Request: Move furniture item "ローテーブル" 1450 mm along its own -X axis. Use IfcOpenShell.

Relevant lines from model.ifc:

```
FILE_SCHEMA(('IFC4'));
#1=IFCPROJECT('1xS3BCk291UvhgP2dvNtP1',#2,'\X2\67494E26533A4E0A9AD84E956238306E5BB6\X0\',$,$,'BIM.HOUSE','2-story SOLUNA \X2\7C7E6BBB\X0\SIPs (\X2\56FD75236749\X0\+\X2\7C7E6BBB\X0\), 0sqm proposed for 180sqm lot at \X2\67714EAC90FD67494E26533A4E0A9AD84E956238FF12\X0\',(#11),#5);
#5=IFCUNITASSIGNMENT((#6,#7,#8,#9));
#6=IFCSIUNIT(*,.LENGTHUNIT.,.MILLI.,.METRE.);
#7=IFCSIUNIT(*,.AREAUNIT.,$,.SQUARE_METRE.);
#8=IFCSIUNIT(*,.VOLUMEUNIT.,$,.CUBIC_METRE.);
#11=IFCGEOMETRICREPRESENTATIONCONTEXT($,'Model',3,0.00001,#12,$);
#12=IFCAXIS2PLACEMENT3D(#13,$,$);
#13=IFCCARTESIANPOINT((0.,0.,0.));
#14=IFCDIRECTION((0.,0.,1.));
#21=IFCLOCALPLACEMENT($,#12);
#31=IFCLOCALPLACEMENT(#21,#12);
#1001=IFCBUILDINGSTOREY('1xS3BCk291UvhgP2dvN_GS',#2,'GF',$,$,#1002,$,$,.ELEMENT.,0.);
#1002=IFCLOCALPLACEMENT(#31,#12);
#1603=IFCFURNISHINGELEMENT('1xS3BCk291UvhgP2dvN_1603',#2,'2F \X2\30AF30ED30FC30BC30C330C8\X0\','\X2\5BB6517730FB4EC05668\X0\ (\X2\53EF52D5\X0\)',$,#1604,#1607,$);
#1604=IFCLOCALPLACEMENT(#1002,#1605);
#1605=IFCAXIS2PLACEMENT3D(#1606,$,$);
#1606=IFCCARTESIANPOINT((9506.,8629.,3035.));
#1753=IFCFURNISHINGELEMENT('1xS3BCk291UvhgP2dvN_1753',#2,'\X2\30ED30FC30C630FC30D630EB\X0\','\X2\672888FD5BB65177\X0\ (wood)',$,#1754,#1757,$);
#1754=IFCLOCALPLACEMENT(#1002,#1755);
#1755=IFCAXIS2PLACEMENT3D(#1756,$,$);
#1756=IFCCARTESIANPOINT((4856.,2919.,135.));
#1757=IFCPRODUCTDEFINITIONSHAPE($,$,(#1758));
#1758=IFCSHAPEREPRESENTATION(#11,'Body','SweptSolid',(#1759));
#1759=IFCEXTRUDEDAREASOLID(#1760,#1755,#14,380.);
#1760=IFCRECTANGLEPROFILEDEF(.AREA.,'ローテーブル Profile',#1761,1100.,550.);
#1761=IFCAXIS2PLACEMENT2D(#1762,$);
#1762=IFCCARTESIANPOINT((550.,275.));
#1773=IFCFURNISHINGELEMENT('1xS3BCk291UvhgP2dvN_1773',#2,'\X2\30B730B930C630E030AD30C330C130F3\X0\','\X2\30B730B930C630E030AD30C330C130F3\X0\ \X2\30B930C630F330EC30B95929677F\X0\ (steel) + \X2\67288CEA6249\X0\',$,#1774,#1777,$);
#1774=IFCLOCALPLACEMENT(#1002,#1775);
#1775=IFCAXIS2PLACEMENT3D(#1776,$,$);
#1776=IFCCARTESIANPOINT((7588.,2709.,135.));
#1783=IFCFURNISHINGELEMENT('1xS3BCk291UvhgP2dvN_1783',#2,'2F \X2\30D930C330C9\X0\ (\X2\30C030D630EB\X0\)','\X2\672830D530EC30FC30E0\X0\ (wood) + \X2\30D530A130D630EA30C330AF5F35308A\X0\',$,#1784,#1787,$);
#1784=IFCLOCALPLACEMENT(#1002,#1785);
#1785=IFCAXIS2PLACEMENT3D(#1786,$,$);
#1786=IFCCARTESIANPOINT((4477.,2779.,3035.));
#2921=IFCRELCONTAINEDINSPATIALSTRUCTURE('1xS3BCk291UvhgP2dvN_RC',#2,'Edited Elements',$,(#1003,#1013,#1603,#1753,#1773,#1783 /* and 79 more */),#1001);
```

```python
import ifcopenshell
import ifcopenshell.api.geometry
import ifcopenshell.util.placement
import ifcopenshell.util.unit

model = ifcopenshell.open("model.ifc")
unit_scale = ifcopenshell.util.unit.calculate_unit_scale(model)

item = model.by_guid("1xS3BCk291UvhgP2dvN_1753")
matrix = ifcopenshell.util.placement.get_local_placement(item.ObjectPlacement)
matrix[:3, 3] -= matrix[:3, 0] * 1.45 / unit_scale
ifcopenshell.api.geometry.edit_object_placement(model, product=item, matrix=matrix, is_si=False)

print(ifcopenshell.util.placement.get_local_placement(item.ObjectPlacement).round(3) + 0.0)

model.write("model_edited.ifc")
```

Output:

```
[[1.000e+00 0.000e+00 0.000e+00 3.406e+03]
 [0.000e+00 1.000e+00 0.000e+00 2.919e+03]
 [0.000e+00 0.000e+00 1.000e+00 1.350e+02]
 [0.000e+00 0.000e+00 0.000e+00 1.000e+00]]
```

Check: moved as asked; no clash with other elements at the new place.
